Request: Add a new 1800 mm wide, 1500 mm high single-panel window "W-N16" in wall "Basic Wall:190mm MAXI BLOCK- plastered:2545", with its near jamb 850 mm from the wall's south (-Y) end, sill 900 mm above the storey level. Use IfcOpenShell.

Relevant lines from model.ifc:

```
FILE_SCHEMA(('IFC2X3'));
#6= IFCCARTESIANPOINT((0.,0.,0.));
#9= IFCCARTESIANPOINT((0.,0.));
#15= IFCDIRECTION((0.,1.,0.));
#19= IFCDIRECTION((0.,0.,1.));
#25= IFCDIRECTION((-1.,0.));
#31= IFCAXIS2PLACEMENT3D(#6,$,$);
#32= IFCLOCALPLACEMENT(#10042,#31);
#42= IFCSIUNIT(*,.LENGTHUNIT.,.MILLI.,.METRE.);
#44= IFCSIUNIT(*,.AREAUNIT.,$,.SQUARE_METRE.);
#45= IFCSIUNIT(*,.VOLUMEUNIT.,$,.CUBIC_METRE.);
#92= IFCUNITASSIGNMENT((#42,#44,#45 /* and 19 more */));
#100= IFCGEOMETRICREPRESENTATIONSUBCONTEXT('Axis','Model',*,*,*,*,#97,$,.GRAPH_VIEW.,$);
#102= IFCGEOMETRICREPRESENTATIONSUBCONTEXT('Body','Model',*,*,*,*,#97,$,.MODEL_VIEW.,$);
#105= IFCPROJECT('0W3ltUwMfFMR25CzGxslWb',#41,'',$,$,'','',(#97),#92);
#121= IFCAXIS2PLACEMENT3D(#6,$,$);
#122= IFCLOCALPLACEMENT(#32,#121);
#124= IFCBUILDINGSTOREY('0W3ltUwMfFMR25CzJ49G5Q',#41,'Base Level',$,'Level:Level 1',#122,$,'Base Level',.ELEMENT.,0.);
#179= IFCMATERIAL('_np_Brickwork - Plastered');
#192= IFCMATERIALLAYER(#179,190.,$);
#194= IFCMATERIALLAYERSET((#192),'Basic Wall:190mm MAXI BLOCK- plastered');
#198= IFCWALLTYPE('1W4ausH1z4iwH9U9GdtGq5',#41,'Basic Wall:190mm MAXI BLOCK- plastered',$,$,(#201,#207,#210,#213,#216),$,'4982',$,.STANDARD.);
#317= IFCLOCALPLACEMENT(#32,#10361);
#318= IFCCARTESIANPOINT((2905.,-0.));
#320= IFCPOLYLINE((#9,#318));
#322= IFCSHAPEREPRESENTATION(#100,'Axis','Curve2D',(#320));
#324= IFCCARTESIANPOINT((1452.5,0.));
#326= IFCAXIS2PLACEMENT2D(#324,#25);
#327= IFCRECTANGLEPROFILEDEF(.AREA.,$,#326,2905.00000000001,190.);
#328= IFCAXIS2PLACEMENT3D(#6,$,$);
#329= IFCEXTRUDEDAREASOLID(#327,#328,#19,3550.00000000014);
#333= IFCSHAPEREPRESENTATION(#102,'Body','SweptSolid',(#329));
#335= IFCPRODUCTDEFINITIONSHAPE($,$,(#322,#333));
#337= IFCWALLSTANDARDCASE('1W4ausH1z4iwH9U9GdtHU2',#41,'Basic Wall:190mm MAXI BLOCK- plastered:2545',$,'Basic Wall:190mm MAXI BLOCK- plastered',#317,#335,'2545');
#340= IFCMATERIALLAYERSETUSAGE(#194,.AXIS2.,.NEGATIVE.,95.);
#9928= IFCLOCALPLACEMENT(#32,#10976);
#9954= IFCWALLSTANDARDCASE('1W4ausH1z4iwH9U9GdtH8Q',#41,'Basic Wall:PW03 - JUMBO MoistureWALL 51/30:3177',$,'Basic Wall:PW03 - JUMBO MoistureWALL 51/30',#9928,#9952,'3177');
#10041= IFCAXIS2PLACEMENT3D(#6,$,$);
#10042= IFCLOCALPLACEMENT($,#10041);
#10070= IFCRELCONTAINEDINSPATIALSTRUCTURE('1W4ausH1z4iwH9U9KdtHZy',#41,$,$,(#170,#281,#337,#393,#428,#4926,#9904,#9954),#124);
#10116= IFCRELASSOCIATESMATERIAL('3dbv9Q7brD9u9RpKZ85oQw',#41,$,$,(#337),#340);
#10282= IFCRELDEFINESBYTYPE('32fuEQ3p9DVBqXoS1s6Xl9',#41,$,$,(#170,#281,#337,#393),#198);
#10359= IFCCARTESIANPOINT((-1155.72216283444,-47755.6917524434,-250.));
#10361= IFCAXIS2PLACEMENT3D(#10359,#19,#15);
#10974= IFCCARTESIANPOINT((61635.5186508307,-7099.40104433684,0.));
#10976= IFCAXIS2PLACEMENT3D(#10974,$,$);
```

```python
import numpy as np
import ifcopenshell
import ifcopenshell.api.feature
import ifcopenshell.api.geometry
import ifcopenshell.api.root
import ifcopenshell.api.spatial
import ifcopenshell.api.type
import ifcopenshell.geom
import ifcopenshell.util.element
import ifcopenshell.util.placement
import ifcopenshell.util.representation
import ifcopenshell.util.shape
import ifcopenshell.util.unit

model = ifcopenshell.open("model.ifc")
unit_scale = ifcopenshell.util.unit.calculate_unit_scale(model)
settings = ifcopenshell.geom.settings()


def volume(element):
    """Net volume in cubic metres, openings subtracted."""
    shape = ifcopenshell.geom.create_shape(settings, element)
    return ifcopenshell.util.shape.get_volume(shape.geometry)


wall = model.by_id(337)
storey = ifcopenshell.util.element.get_container(wall, ifc_class="IfcBuildingStorey")
context = ifcopenshell.util.representation.get_context(model, "Model", "Body", "MODEL_VIEW")
before = volume(wall)

width, height, from_end, sill = 1.8, 1.5, 0.85, 0.9  # metres

# The wall runs along its own X axis, and the end named is its -X end.
wall_shape = ifcopenshell.geom.create_shape(settings, wall)
x, y, z = ifcopenshell.util.shape.get_vertices(wall_shape.geometry).T
start = x.min() + from_end
face, thickness = float(y.min()), float(y.max() - y.min())
wall_matrix = ifcopenshell.util.placement.get_local_placement(wall.ObjectPlacement)
level = ifcopenshell.util.placement.get_local_placement(storey.ObjectPlacement)[2, 3]


def in_wall(x, y):
    """Placement at x, y metres in the wall's axes, at sill height."""
    matrix = wall_matrix.copy()
    matrix[:, 3] = wall_matrix @ np.array([x / unit_scale, y / unit_scale, 0.0, 1.0])
    matrix[2, 3] = level + sill / unit_scale
    return matrix


# Opening: a box that overshoots both wall faces by 50 mm.
opening = ifcopenshell.api.root.create_entity(model, ifc_class="IfcOpeningElement")
box = ifcopenshell.api.geometry.add_wall_representation(
    model, context=context, length=width, height=height, thickness=thickness + 0.1
)
ifcopenshell.api.geometry.assign_representation(model, product=opening, representation=box)
ifcopenshell.api.geometry.edit_object_placement(model, product=opening, matrix=in_wall(start, face - 0.05), is_si=False)
ifcopenshell.api.feature.add_feature(model, feature=opening, element=wall)

window = ifcopenshell.api.root.create_entity(model, ifc_class="IfcWindow", name="W-N16")
window.OverallWidth, window.OverallHeight = width / unit_scale, height / unit_scale
body = ifcopenshell.api.geometry.add_window_representation(
    model,
    context=context,
    overall_width=window.OverallWidth,
    overall_height=window.OverallHeight,
    partition_type="SINGLE_PANEL",
)
ifcopenshell.api.geometry.assign_representation(model, product=window, representation=body)
ifcopenshell.api.spatial.assign_container(model, products=[window], relating_structure=storey)
fills = ifcopenshell.api.feature.add_filling(model, opening=opening, element=window)
fills.OwnerHistory = window.OwnerHistory  # required in IFC2X3

# IFC2X3 keeps the operation on the window style.
style = ifcopenshell.api.root.create_entity(model, ifc_class="IfcWindowStyle", name="W-N16")
style.OperationType, style.ConstructionType = "SINGLE_PANEL", "NOTDEFINED"
style.ParameterTakesPrecedence = style.Sizeable = False
ifcopenshell.api.type.assign_type(model, related_objects=[window], relating_type=style)

# Centre the window in the wall's thickness.
ifcopenshell.api.geometry.edit_object_placement(model, product=window, matrix=in_wall(start, face), is_si=False)
window_shape = ifcopenshell.geom.create_shape(settings, window)
depth = ifcopenshell.util.shape.get_vertices(window_shape.geometry)[:, 1]
offset = face + thickness / 2 - (depth.min() + depth.max()) / 2
ifcopenshell.api.geometry.edit_object_placement(model, product=window, matrix=in_wall(start, offset), is_si=False)

after = volume(wall)

print(f"wall volume {before:.3f} -> {after:.3f} m3")

model.write("model_v2.ifc")
```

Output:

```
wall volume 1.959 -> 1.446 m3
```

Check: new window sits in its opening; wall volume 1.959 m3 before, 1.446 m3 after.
